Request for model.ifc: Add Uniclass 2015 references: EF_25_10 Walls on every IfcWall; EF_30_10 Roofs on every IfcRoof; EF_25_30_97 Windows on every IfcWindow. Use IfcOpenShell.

First a look at what the model holds.

```python
import ifcopenshell

model = ifcopenshell.open("model.ifc")
print(model.schema)
print("classifications:", [c.Name for c in model.by_type("IfcClassification")])
for ifc_class in ("IfcDoor", "IfcRoof", "IfcStair", "IfcWall", "IfcWindow"):
    print(ifc_class, len(model.by_type(ifc_class)))
```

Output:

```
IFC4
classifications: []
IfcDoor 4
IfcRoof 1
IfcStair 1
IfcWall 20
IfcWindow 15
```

```python
import ifcopenshell
import ifcopenshell.api.classification

model = ifcopenshell.open("model.ifc")

system = ifcopenshell.api.classification.add_classification(model, classification="Uniclass 2015")

codes = {
    "IfcWall": ("EF_25_10", "Walls"),
    "IfcRoof": ("EF_30_10", "Roofs"),
    "IfcWindow": ("EF_25_30_97", "Windows"),
}
for ifc_class, (code, name) in codes.items():
    products = model.by_type(ifc_class)
    ifcopenshell.api.classification.add_reference(
        model, products=products, classification=system, identification=code, name=name
    )
    print(code, len(products))

model.write("model-out.ifc")
```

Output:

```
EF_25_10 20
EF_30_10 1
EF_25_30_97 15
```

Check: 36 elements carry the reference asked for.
